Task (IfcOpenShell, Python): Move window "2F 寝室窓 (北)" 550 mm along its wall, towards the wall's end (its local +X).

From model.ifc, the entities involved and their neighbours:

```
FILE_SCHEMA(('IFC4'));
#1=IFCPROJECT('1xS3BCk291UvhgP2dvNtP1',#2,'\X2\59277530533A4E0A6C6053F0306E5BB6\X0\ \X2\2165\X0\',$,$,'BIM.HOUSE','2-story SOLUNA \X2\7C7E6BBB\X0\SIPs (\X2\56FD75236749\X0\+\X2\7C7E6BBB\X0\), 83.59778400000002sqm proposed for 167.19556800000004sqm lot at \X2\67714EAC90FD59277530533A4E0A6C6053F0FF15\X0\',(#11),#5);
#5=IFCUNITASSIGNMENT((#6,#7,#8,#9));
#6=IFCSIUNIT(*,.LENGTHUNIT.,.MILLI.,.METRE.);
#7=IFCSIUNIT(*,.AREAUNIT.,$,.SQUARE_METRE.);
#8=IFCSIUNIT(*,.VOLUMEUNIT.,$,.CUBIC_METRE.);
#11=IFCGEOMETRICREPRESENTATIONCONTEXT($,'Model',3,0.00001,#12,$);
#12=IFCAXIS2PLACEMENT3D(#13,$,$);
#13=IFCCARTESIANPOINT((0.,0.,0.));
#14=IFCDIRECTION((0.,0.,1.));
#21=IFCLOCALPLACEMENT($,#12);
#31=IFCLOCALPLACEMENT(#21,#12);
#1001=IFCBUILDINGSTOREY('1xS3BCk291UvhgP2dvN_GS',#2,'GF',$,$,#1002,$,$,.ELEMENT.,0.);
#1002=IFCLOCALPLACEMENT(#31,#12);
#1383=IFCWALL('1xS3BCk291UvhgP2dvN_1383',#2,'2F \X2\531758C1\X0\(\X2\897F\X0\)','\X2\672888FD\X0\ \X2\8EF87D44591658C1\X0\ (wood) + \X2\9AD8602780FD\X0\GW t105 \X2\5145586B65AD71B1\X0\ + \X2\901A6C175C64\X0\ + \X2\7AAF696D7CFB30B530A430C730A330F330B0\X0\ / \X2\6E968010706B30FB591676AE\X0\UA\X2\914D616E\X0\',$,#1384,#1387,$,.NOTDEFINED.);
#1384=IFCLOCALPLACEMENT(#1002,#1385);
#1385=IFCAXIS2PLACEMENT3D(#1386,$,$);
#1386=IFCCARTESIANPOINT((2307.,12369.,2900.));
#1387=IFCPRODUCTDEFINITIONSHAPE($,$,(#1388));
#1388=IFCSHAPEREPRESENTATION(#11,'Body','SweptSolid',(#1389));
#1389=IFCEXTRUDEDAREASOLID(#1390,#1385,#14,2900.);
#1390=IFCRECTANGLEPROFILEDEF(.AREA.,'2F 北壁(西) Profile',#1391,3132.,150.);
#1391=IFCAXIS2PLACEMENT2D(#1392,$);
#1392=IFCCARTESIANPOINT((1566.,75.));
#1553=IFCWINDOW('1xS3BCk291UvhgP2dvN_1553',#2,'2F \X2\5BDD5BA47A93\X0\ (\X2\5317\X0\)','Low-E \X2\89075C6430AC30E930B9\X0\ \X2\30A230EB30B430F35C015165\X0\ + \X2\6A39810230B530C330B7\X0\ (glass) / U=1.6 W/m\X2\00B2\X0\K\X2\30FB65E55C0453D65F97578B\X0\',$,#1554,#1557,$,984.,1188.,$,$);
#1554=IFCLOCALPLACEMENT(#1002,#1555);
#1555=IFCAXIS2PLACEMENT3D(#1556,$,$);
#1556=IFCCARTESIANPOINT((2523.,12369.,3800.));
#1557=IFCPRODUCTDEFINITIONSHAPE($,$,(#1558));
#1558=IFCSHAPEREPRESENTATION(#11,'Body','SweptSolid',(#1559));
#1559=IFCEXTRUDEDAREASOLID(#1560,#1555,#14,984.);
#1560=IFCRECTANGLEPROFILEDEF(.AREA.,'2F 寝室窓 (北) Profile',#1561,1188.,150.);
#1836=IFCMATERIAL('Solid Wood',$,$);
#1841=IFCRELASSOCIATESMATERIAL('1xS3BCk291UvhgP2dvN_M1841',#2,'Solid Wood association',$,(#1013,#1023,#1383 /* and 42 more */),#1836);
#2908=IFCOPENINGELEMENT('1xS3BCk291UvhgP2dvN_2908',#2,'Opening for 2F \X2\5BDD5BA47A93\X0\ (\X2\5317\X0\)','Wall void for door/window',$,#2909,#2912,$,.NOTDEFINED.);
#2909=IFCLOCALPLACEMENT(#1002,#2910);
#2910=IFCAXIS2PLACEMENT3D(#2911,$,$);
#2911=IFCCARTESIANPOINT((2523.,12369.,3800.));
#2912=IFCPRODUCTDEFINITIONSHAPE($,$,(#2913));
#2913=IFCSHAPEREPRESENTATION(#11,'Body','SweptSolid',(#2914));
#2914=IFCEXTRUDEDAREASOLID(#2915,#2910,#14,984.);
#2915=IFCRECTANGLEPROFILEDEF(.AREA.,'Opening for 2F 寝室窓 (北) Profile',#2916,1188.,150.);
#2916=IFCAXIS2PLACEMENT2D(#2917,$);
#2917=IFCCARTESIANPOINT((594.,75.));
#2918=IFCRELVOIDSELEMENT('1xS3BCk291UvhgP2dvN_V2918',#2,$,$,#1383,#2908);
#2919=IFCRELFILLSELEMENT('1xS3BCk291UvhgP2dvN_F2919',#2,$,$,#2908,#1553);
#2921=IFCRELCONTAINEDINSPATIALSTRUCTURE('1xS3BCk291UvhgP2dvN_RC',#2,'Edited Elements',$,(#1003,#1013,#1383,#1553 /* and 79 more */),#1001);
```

```python
import ifcopenshell
import ifcopenshell.api.geometry
import ifcopenshell.util.placement

model = ifcopenshell.open("model.ifc")

window = model.by_id(1553)
opening = window.FillsVoids[0].RelatingOpeningElement
wall = opening.VoidsElements[0].RelatingBuildingElement

wall_matrix = ifcopenshell.util.placement.get_local_placement(wall.ObjectPlacement)
shift = wall_matrix[:3, 0] * 550.0
before = ifcopenshell.util.placement.get_local_placement(window.ObjectPlacement)[:3, 3].copy()

# The window is not placed relative to its opening, so move both.
for product in (opening, window):
    matrix = ifcopenshell.util.placement.get_local_placement(product.ObjectPlacement)
    matrix[:3, 3] += shift
    ifcopenshell.api.geometry.edit_object_placement(model, product=product, matrix=matrix, is_si=False)

after = ifcopenshell.util.placement.get_local_placement(window.ObjectPlacement)[:3, 3]
print("window moved by", (after - before).round(3) + 0.0)

model.write("model_updated.ifc")
```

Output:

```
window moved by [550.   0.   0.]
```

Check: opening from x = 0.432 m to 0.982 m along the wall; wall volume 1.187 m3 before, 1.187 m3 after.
